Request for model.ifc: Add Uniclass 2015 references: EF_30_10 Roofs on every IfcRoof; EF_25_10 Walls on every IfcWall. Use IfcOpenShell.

First a look at what the model holds.

```python
import ifcopenshell

model = ifcopenshell.open("model.ifc")
print(model.schema)
print("classifications:", [c.Name for c in model.by_type("IfcClassification")])
for ifc_class in ("IfcDoor", "IfcRoof", "IfcStair", "IfcWall", "IfcWindow"):
    print(ifc_class, len(model.by_type(ifc_class)))
```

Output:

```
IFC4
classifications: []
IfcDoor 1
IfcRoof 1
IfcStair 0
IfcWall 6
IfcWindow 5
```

```python
import ifcopenshell
import ifcopenshell.api.classification

model = ifcopenshell.open("model.ifc")

system = ifcopenshell.api.classification.add_classification(model, classification="Uniclass 2015")

codes = {
    "IfcRoof": ("EF_30_10", "Roofs"),
    "IfcWall": ("EF_25_10", "Walls"),
}
for ifc_class, (code, name) in codes.items():
    products = model.by_type(ifc_class)
    ifcopenshell.api.classification.add_reference(
        model, products=products, classification=system, identification=code, name=name
    )
    print(code, len(products))

model.write("model_v2.ifc")
```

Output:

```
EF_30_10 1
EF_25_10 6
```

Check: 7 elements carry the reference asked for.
